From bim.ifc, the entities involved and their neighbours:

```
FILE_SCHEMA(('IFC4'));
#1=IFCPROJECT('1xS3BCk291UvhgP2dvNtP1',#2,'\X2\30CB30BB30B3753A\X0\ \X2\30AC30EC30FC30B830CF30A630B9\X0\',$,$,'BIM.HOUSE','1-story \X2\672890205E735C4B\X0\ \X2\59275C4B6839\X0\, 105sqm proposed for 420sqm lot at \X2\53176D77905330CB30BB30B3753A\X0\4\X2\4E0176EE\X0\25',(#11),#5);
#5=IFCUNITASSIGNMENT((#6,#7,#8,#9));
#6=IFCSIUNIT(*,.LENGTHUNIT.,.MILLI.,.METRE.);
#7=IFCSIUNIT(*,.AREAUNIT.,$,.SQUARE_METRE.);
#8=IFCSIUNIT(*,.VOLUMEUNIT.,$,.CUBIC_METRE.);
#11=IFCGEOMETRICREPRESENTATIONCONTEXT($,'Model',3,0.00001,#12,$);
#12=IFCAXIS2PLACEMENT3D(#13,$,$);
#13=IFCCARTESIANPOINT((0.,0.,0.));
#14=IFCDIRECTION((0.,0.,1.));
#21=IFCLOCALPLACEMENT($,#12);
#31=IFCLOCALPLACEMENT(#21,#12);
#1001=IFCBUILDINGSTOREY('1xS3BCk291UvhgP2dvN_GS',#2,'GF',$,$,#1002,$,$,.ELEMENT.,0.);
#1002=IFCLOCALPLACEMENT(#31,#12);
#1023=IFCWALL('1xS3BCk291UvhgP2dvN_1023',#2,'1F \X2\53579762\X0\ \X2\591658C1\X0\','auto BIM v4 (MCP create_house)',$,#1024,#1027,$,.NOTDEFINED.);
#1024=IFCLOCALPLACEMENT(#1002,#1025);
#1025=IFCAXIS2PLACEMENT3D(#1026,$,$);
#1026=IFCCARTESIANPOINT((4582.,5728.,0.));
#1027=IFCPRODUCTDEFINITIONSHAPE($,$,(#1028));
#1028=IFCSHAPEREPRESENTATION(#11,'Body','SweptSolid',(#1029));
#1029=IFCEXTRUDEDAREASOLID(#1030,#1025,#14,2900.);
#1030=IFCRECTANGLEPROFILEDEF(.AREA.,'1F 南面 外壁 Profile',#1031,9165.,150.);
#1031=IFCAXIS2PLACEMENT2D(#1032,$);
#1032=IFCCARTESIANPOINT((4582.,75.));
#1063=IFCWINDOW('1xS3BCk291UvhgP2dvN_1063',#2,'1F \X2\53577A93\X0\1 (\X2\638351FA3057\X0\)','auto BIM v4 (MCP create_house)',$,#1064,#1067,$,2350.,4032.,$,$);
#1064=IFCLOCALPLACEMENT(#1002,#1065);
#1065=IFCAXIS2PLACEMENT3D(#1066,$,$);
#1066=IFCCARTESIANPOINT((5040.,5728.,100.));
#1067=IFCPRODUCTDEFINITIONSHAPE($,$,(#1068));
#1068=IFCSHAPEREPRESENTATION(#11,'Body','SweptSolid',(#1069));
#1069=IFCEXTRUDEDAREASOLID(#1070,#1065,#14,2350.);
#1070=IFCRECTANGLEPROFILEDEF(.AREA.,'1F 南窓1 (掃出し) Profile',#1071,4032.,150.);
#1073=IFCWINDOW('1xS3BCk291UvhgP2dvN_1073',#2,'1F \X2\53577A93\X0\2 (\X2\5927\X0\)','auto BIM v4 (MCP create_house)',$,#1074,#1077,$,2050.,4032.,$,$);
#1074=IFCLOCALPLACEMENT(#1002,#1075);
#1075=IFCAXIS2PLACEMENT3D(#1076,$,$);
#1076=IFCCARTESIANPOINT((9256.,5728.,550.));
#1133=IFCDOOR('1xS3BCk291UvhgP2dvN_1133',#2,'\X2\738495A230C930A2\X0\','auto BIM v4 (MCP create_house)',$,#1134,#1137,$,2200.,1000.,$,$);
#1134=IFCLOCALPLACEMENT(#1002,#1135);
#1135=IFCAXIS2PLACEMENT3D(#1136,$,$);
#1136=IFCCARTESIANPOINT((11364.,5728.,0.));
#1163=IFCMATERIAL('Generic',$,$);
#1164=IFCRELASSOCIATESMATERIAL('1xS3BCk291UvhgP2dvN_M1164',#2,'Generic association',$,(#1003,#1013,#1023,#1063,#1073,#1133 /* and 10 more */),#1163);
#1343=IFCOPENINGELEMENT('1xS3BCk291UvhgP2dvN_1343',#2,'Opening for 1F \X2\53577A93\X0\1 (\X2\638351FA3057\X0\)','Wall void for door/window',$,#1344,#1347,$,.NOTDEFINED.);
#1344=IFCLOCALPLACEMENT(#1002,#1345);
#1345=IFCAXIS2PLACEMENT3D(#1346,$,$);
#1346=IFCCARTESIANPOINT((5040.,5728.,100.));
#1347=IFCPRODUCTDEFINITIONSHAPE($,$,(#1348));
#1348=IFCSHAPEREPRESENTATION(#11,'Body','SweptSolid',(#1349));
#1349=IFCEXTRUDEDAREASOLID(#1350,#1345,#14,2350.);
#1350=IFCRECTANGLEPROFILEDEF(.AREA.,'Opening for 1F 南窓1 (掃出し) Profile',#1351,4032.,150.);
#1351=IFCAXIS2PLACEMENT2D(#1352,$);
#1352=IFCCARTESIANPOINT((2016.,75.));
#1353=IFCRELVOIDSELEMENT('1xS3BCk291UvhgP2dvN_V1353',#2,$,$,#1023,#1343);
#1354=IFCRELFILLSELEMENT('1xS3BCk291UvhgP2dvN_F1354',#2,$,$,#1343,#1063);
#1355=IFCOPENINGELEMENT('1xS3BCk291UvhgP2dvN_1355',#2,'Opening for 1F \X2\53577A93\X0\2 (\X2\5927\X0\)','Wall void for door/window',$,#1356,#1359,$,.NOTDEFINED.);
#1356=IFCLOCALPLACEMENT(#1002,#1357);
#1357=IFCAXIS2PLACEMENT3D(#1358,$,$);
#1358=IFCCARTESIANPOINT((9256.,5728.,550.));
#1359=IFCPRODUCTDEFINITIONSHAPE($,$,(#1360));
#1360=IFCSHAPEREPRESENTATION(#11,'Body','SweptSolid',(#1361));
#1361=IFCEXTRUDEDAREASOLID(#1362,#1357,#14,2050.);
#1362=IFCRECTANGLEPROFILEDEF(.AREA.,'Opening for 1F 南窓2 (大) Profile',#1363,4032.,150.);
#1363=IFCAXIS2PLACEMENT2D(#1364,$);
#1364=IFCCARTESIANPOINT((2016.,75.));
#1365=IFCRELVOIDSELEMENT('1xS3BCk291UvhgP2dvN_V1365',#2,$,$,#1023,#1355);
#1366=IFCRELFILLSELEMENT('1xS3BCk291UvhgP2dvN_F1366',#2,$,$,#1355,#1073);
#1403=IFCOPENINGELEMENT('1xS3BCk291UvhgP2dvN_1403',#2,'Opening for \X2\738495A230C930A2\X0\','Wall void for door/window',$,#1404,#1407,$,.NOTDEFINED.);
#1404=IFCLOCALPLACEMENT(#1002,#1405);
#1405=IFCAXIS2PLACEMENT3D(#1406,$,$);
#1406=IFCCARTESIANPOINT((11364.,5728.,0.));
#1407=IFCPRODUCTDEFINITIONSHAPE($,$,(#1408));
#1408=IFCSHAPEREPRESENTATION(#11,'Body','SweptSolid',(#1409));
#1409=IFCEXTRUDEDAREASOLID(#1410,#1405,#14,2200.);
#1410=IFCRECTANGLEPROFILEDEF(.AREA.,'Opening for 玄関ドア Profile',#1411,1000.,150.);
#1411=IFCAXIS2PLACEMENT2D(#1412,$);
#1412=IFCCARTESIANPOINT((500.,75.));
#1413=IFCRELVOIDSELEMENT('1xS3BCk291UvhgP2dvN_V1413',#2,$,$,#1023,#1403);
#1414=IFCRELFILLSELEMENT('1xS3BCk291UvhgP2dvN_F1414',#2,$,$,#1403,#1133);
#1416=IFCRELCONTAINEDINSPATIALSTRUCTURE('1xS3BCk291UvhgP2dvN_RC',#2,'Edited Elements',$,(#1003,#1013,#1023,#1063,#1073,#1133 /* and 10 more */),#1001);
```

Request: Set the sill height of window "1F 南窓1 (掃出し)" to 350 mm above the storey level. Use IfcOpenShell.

```python
import numpy as np
import ifcopenshell
import ifcopenshell.api.geometry
import ifcopenshell.geom
import ifcopenshell.util.element
import ifcopenshell.util.placement
import ifcopenshell.util.shape
import ifcopenshell.util.unit

model = ifcopenshell.open("bim.ifc")
unit_scale = ifcopenshell.util.unit.calculate_unit_scale(model)

window = model.by_id(1063)
opening = window.FillsVoids[0].RelatingOpeningElement
storey = ifcopenshell.util.element.get_container(window, ifc_class="IfcBuildingStorey")
level = ifcopenshell.util.placement.get_local_placement(storey.ObjectPlacement)[2, 3]

# The opening's origin need not be at the sill, so measure its lowest point.
shape = ifcopenshell.geom.create_shape(ifcopenshell.geom.settings(), opening)
bottom = ifcopenshell.util.shape.get_shape_bottom_elevation(shape, shape.geometry) / unit_scale
dz = level + 350.0 - bottom

shift = np.array([0.0, 0.0, dz])
# The window is not placed relative to its opening, so move both.
for product in (opening, window):
    matrix = ifcopenshell.util.placement.get_local_placement(product.ObjectPlacement)
    matrix[:3, 3] += shift
    ifcopenshell.api.geometry.edit_object_placement(model, product=product, matrix=matrix, is_si=False)

print(f"moved by {dz * unit_scale:+.3f} m")

model.write("bim_v2.ifc")
```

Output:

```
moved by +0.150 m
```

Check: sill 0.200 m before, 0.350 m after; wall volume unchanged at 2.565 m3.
